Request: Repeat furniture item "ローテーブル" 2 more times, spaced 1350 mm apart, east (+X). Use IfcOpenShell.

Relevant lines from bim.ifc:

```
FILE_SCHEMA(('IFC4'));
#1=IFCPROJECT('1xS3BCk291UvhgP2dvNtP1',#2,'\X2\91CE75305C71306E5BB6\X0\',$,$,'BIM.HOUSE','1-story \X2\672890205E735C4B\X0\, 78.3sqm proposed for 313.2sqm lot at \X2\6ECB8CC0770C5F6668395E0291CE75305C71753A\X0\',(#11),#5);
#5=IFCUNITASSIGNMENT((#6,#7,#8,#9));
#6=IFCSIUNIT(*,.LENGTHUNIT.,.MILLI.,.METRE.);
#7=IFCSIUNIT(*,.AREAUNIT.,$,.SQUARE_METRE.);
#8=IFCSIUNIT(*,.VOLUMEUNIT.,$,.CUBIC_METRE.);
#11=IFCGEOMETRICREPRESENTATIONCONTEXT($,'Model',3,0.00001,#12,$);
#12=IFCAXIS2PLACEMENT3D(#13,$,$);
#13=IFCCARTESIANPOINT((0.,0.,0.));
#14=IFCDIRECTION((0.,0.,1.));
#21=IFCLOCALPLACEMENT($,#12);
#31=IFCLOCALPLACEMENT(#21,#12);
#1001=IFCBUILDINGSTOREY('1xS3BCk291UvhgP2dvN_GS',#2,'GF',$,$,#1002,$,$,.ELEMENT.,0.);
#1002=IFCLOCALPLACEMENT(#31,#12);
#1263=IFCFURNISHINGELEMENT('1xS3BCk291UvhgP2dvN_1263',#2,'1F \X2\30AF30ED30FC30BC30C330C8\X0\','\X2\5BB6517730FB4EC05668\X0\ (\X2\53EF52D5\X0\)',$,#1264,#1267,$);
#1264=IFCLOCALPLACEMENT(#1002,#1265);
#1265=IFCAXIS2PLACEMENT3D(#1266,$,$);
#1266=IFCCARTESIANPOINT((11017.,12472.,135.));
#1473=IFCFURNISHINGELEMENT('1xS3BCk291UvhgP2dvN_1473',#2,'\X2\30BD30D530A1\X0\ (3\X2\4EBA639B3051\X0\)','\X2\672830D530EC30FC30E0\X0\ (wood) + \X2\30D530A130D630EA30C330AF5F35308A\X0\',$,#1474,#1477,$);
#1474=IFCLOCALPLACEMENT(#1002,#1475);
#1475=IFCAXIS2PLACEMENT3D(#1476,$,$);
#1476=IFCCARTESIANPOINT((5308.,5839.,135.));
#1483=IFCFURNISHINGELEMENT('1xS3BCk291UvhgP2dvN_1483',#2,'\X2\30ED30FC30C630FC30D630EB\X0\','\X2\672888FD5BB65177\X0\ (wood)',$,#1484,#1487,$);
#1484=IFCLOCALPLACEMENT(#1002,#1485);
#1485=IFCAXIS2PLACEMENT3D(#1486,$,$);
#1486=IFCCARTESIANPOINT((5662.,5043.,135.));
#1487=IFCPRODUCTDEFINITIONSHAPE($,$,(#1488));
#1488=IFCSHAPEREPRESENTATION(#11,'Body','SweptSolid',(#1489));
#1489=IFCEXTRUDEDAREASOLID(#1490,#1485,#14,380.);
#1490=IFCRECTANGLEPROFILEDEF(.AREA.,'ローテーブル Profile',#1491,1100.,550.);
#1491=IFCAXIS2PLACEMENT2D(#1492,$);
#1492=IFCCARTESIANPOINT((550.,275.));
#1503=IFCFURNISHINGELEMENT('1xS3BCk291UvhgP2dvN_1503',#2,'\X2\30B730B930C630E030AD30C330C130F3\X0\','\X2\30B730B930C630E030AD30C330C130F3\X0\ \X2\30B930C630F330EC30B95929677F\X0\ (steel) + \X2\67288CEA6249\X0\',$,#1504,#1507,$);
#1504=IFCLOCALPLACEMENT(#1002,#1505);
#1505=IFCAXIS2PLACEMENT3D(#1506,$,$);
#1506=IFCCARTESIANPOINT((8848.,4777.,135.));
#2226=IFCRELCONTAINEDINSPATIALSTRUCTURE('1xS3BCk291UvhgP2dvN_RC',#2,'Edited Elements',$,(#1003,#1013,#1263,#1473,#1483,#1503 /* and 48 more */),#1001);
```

```python
import numpy as np
import ifcopenshell
import ifcopenshell.api.geometry
import ifcopenshell.api.root
import ifcopenshell.util.element
import ifcopenshell.util.placement

model = ifcopenshell.open("bim.ifc")


def reuse_history(source, copy):
    """copy_class also copies each property set's owner history, people and application; keep the originals."""
    for rel in copy.IsDefinedBy:
        if rel.is_a("IfcRelDefinesByProperties") and (history := rel.RelatingPropertyDefinition.OwnerHistory):
            rel.RelatingPropertyDefinition.OwnerHistory = source.OwnerHistory
            ifcopenshell.util.element.remove_deep2(model, history)


source = model.by_id(1483)
base = ifcopenshell.util.placement.get_local_placement(source.ObjectPlacement)
step = np.array([1.0, 0.0, 0.0]) * 1350.0

for i in range(1, 3):
    copy = ifcopenshell.api.root.copy_class(model, product=source)
    copy.Representation = ifcopenshell.util.element.copy_deep(
        model, source.Representation, exclude=["IfcGeometricRepresentationContext", "IfcRepresentationMap"]
    )
    reuse_history(source, copy)
    matrix = base.copy()
    matrix[:3, 3] += i * step
    print("added at", matrix[:3, 3].round(3) + 0.0)
    ifcopenshell.api.geometry.edit_object_placement(model, product=copy, matrix=matrix, is_si=False)

model.write("bim_rev.ifc")
```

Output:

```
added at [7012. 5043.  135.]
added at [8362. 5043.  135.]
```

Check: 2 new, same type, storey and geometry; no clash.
